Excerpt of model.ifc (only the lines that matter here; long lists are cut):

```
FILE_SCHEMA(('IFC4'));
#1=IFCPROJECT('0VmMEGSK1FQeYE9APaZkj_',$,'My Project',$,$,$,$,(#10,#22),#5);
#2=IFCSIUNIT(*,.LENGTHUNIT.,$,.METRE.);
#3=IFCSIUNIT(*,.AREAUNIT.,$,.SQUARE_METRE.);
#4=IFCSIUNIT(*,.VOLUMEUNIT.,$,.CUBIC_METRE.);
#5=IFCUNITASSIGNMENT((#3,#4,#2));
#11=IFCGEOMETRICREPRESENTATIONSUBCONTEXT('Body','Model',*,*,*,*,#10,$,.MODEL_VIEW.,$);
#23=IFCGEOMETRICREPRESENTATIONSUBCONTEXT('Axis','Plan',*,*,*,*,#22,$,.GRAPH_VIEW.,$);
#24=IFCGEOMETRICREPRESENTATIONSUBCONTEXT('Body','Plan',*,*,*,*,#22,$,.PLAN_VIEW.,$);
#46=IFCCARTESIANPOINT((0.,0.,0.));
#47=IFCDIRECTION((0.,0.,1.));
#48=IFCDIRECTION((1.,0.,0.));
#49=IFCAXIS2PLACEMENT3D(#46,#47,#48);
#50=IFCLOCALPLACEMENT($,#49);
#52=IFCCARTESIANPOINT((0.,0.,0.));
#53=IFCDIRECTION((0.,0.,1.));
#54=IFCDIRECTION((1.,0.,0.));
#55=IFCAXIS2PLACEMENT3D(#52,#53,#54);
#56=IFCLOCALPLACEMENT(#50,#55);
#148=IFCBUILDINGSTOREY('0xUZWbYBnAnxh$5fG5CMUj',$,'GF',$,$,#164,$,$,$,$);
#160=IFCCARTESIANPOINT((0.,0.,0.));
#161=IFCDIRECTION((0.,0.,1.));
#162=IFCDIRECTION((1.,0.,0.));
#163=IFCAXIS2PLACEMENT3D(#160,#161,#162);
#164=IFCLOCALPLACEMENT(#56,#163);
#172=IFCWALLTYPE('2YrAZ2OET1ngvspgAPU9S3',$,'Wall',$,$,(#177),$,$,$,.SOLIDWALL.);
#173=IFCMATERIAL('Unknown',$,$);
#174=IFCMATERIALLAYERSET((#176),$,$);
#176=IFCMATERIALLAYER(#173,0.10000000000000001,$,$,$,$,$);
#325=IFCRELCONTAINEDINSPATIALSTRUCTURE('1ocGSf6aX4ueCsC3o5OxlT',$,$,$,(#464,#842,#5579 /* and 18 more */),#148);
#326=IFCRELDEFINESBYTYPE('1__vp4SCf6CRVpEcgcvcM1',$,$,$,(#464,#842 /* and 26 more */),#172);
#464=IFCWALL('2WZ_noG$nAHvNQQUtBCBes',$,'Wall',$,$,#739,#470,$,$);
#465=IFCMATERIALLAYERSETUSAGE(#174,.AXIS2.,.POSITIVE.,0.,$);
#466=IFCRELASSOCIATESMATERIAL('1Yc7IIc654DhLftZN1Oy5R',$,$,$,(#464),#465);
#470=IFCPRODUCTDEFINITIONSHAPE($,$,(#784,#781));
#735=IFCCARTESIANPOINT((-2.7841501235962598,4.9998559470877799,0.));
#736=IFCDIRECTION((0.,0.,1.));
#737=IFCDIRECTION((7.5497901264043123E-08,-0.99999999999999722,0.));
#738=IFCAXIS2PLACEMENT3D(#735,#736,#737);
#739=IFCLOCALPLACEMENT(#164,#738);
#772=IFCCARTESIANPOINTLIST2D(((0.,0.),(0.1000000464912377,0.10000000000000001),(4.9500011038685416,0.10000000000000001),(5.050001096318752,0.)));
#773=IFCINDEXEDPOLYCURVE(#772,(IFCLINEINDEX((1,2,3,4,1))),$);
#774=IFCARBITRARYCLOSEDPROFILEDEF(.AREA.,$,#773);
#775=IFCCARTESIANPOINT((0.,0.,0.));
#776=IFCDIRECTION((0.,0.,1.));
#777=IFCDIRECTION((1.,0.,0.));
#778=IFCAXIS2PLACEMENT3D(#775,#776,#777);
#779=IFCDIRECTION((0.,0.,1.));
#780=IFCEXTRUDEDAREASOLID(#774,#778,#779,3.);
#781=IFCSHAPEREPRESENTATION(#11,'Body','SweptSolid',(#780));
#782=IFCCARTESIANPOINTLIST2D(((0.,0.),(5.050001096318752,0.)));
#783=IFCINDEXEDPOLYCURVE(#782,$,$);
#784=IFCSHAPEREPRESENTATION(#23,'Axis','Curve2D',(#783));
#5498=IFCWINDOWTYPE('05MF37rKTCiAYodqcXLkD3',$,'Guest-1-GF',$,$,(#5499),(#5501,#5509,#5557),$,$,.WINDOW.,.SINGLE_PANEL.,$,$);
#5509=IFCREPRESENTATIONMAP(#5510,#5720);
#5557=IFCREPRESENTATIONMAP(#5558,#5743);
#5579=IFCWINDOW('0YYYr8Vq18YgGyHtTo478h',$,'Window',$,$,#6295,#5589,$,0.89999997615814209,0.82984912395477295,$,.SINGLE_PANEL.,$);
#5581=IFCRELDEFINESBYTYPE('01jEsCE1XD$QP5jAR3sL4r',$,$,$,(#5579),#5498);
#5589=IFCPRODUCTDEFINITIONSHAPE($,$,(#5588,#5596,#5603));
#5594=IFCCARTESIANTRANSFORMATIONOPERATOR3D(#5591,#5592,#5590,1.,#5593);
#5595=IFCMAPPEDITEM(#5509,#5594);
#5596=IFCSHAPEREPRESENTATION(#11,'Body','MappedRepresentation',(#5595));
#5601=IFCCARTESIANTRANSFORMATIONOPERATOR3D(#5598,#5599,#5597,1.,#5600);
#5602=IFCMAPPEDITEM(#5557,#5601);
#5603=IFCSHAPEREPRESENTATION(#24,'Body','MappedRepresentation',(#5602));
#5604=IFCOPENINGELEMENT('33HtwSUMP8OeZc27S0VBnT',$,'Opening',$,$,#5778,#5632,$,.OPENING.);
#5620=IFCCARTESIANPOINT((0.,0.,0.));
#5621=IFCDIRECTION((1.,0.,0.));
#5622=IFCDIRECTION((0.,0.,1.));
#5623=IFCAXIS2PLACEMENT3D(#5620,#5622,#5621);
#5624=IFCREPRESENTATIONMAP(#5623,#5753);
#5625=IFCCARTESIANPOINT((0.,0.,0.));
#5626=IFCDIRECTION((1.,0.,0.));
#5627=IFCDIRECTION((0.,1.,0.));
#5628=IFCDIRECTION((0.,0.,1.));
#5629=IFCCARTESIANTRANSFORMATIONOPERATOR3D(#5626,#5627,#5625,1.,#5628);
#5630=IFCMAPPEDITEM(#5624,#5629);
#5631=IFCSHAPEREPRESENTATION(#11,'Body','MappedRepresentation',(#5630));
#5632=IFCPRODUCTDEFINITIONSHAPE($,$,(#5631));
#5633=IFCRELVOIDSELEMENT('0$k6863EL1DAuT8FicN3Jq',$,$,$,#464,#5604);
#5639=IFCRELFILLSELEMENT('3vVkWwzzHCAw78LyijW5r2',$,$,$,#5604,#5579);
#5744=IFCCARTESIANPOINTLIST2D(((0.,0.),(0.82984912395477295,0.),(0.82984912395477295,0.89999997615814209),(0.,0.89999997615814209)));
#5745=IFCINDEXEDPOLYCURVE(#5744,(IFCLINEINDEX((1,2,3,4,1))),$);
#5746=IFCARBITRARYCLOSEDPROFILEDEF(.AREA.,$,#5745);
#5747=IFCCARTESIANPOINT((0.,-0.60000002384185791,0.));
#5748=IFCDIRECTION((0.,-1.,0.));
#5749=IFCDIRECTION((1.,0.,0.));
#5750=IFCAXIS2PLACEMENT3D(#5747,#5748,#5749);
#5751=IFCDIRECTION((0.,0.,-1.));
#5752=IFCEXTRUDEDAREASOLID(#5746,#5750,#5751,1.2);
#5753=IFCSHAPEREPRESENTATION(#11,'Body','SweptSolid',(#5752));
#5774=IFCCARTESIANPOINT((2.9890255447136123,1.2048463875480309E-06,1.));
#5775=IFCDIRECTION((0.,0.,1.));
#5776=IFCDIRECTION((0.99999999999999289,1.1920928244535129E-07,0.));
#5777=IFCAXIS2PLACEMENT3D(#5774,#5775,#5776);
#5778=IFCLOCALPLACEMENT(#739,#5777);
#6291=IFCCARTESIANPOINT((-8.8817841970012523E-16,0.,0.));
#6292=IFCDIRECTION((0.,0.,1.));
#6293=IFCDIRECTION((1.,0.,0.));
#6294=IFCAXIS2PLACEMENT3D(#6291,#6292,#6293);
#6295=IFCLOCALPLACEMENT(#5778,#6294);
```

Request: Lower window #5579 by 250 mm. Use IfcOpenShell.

```python
import numpy as np
import ifcopenshell
import ifcopenshell.api.geometry
import ifcopenshell.util.placement
import ifcopenshell.util.unit

model = ifcopenshell.open("model.ifc")
unit_scale = ifcopenshell.util.unit.calculate_unit_scale(model)

window = model.by_guid("0YYYr8Vq18YgGyHtTo478h")
opening = window.FillsVoids[0].RelatingOpeningElement
dz = -0.25 / unit_scale

shift = np.array([0.0, 0.0, dz])
# The window is placed relative to its opening, so it follows when the opening moves.
matrix = ifcopenshell.util.placement.get_local_placement(opening.ObjectPlacement)
matrix[:3, 3] += shift
ifcopenshell.api.geometry.edit_object_placement(
    model, product=opening, matrix=matrix, is_si=False, should_transform_children=True
)

print(f"moved by {dz * unit_scale:+.3f} m")

model.write("model_edited.ifc")
```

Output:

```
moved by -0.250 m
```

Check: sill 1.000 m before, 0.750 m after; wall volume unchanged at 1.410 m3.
